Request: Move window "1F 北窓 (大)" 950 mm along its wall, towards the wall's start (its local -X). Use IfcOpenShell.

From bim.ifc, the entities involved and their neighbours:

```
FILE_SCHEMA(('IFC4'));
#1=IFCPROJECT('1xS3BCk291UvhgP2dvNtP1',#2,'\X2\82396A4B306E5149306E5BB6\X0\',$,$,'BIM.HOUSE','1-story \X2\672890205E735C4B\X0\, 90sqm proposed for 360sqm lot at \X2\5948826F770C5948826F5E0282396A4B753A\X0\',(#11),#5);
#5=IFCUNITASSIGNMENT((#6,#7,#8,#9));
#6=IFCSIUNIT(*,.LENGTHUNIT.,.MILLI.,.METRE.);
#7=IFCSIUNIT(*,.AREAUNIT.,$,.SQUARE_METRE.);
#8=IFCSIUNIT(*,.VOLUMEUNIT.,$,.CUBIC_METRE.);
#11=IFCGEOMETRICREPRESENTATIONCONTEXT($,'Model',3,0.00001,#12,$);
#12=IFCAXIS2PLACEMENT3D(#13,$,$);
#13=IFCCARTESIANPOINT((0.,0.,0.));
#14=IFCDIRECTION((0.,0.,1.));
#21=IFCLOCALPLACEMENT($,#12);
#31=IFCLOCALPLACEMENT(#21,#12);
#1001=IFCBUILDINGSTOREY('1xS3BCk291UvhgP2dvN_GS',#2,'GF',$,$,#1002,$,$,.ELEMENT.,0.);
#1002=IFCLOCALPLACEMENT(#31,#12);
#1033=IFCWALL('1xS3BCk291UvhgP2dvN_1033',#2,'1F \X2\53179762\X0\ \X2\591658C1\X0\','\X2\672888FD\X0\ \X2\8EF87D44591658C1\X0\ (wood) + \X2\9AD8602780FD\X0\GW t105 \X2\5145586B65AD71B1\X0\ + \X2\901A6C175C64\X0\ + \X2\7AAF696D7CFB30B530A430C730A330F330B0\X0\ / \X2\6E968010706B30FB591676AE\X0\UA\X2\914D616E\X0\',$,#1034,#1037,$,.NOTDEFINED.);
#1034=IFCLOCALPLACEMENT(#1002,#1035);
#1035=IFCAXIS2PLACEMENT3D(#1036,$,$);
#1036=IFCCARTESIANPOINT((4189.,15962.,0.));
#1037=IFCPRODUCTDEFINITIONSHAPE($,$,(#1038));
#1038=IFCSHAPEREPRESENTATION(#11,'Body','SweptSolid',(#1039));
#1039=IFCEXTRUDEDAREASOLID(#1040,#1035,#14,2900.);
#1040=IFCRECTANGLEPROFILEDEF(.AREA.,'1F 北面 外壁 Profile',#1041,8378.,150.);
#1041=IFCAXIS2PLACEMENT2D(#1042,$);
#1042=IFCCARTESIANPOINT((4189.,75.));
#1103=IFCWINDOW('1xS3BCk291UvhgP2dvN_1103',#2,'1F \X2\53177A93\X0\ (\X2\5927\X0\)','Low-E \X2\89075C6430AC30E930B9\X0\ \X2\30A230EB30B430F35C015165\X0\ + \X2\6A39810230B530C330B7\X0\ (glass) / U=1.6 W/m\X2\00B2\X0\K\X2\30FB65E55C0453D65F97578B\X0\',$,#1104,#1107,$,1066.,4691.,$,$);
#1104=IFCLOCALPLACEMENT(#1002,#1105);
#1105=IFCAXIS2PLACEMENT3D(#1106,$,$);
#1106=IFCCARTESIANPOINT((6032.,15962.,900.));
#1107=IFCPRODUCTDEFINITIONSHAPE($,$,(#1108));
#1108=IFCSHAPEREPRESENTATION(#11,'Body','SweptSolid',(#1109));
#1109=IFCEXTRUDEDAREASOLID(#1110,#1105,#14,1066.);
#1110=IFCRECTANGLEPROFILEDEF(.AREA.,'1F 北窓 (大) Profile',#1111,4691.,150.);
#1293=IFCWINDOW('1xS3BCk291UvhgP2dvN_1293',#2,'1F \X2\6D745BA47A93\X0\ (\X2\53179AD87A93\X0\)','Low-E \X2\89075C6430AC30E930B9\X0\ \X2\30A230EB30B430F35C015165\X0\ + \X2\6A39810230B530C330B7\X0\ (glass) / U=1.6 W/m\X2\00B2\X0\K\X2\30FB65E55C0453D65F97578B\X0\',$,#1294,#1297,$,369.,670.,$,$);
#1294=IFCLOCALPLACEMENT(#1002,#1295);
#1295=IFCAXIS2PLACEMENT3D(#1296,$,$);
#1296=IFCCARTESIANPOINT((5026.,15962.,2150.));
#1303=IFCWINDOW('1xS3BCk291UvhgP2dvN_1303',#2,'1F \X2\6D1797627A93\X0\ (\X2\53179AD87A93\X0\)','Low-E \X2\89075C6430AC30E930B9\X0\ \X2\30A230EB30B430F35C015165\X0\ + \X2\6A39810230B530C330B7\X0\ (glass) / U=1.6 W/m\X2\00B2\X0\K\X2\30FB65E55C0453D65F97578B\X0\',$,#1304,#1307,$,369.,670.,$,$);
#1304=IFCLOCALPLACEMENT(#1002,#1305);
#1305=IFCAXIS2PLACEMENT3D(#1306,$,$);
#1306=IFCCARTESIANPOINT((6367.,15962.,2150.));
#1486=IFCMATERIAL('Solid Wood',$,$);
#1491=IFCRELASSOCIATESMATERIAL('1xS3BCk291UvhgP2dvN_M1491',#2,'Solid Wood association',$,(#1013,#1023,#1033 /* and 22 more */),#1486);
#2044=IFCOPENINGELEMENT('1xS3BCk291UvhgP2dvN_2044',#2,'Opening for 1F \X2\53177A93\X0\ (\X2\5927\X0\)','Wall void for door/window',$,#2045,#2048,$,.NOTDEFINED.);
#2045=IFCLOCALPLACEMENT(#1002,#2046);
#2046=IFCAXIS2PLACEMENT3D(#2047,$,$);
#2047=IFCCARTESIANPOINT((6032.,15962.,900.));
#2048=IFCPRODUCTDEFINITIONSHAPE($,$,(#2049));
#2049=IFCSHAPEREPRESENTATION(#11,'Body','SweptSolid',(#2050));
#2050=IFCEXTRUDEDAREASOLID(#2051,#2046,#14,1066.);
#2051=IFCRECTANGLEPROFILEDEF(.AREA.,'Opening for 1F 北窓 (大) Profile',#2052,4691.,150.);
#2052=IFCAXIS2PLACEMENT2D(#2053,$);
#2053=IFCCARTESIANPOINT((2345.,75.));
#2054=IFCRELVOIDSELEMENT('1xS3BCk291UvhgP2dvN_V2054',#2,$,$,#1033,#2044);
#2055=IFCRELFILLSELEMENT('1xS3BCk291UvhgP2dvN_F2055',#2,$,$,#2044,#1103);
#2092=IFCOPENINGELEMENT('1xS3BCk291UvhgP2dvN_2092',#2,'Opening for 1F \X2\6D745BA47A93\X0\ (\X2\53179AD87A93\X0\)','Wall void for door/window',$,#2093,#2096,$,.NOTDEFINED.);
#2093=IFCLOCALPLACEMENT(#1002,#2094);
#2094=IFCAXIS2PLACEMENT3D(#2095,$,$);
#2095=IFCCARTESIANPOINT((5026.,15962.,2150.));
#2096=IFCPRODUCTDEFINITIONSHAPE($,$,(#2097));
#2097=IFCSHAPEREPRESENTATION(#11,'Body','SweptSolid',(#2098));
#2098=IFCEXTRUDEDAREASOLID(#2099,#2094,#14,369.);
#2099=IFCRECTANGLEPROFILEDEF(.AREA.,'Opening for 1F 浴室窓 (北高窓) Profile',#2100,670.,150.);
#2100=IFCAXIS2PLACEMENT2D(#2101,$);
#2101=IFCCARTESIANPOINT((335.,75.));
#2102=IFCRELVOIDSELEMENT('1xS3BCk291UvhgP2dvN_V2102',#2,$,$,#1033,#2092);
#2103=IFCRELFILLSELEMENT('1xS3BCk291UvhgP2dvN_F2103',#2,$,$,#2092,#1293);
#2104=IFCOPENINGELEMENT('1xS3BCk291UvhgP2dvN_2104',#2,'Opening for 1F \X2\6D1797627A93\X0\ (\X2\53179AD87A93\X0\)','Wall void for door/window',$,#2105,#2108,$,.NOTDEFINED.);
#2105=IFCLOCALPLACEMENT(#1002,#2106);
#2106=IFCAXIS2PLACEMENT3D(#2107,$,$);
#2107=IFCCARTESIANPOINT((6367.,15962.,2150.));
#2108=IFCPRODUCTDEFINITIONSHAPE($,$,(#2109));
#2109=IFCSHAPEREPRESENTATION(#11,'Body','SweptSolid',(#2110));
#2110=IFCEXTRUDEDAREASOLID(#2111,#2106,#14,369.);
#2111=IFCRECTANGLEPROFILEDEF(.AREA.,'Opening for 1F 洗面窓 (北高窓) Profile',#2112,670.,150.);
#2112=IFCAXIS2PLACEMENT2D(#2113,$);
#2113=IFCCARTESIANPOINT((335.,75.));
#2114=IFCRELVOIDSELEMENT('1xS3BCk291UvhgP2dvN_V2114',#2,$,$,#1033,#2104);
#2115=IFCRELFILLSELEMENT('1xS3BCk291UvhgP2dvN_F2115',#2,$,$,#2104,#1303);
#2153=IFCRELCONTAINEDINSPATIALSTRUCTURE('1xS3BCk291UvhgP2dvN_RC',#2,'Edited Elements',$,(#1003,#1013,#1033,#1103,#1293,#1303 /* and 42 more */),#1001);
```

```python
import ifcopenshell
import ifcopenshell.api.geometry
import ifcopenshell.util.placement
import ifcopenshell.util.unit

model = ifcopenshell.open("bim.ifc")
unit_scale = ifcopenshell.util.unit.calculate_unit_scale(model)

window = model.by_id(1103)
opening = window.FillsVoids[0].RelatingOpeningElement
wall = opening.VoidsElements[0].RelatingBuildingElement

wall_matrix = ifcopenshell.util.placement.get_local_placement(wall.ObjectPlacement)
shift = wall_matrix[:3, 0] * -0.95 / unit_scale
before = ifcopenshell.util.placement.get_local_placement(window.ObjectPlacement)[:3, 3].copy()

# The window is not placed relative to its opening, so move both.
for product in (opening, window):
    matrix = ifcopenshell.util.placement.get_local_placement(product.ObjectPlacement)
    matrix[:3, 3] += shift
    ifcopenshell.api.geometry.edit_object_placement(model, product=product, matrix=matrix, is_si=False)

after = ifcopenshell.util.placement.get_local_placement(window.ObjectPlacement)[:3, 3]
print("window moved by", (after - before).round(3) + 0.0)

model.write("bim_v2.ifc")
```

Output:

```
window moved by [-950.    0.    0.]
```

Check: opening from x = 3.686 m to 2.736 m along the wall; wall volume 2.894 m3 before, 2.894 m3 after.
